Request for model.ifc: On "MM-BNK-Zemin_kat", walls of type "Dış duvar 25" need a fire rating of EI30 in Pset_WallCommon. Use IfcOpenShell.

First a look at what the model holds.

```python
import ifcopenshell
import ifcopenshell.util.element

model = ifcopenshell.open("model.ifc")
print(model.schema)
storey = next(s for s in model.by_type("IfcBuildingStorey") if s.Name == "MM-BNK-Zemin_kat")
walls = [e for e in ifcopenshell.util.element.get_decomposition(storey) if e.is_a("IfcWall")]
seen = {}
for e in walls:
    element_type = ifcopenshell.util.element.get_type(e)
    key = (element_type.Name if element_type != e and element_type else None, ifcopenshell.util.element.get_pset(e, "Pset_WallCommon", "FireRating"))
    seen[key] = seen.get(key, 0) + 1
for (name, value), count in sorted(seen.items(), key=str):
    print(count, "x", name, "|", value)
```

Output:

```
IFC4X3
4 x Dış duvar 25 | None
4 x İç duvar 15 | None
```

```python
import ifcopenshell
import ifcopenshell.api.pset
import ifcopenshell.util.element

model = ifcopenshell.open("model.ifc")

storey = next(s for s in model.by_type("IfcBuildingStorey") if s.Name == "MM-BNK-Zemin_kat")
walls = [e for e in ifcopenshell.util.element.get_decomposition(storey) if e.is_a("IfcWall")]

count = 0
for e in walls:
    element_type = ifcopenshell.util.element.get_type(e)
    if element_type in (None, e) or element_type.Name != "Dış duvar 25":
        continue
    # add_pset returns the element's existing set when there is one.
    pset = ifcopenshell.api.pset.add_pset(model, product=e, name="Pset_WallCommon")
    ifcopenshell.api.pset.edit_pset(model, pset=pset, properties={"FireRating": "EI30"})
    count += 1

print(count, "walls updated")

model.write("model_edited.ifc")
```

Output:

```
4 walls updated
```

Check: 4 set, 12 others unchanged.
